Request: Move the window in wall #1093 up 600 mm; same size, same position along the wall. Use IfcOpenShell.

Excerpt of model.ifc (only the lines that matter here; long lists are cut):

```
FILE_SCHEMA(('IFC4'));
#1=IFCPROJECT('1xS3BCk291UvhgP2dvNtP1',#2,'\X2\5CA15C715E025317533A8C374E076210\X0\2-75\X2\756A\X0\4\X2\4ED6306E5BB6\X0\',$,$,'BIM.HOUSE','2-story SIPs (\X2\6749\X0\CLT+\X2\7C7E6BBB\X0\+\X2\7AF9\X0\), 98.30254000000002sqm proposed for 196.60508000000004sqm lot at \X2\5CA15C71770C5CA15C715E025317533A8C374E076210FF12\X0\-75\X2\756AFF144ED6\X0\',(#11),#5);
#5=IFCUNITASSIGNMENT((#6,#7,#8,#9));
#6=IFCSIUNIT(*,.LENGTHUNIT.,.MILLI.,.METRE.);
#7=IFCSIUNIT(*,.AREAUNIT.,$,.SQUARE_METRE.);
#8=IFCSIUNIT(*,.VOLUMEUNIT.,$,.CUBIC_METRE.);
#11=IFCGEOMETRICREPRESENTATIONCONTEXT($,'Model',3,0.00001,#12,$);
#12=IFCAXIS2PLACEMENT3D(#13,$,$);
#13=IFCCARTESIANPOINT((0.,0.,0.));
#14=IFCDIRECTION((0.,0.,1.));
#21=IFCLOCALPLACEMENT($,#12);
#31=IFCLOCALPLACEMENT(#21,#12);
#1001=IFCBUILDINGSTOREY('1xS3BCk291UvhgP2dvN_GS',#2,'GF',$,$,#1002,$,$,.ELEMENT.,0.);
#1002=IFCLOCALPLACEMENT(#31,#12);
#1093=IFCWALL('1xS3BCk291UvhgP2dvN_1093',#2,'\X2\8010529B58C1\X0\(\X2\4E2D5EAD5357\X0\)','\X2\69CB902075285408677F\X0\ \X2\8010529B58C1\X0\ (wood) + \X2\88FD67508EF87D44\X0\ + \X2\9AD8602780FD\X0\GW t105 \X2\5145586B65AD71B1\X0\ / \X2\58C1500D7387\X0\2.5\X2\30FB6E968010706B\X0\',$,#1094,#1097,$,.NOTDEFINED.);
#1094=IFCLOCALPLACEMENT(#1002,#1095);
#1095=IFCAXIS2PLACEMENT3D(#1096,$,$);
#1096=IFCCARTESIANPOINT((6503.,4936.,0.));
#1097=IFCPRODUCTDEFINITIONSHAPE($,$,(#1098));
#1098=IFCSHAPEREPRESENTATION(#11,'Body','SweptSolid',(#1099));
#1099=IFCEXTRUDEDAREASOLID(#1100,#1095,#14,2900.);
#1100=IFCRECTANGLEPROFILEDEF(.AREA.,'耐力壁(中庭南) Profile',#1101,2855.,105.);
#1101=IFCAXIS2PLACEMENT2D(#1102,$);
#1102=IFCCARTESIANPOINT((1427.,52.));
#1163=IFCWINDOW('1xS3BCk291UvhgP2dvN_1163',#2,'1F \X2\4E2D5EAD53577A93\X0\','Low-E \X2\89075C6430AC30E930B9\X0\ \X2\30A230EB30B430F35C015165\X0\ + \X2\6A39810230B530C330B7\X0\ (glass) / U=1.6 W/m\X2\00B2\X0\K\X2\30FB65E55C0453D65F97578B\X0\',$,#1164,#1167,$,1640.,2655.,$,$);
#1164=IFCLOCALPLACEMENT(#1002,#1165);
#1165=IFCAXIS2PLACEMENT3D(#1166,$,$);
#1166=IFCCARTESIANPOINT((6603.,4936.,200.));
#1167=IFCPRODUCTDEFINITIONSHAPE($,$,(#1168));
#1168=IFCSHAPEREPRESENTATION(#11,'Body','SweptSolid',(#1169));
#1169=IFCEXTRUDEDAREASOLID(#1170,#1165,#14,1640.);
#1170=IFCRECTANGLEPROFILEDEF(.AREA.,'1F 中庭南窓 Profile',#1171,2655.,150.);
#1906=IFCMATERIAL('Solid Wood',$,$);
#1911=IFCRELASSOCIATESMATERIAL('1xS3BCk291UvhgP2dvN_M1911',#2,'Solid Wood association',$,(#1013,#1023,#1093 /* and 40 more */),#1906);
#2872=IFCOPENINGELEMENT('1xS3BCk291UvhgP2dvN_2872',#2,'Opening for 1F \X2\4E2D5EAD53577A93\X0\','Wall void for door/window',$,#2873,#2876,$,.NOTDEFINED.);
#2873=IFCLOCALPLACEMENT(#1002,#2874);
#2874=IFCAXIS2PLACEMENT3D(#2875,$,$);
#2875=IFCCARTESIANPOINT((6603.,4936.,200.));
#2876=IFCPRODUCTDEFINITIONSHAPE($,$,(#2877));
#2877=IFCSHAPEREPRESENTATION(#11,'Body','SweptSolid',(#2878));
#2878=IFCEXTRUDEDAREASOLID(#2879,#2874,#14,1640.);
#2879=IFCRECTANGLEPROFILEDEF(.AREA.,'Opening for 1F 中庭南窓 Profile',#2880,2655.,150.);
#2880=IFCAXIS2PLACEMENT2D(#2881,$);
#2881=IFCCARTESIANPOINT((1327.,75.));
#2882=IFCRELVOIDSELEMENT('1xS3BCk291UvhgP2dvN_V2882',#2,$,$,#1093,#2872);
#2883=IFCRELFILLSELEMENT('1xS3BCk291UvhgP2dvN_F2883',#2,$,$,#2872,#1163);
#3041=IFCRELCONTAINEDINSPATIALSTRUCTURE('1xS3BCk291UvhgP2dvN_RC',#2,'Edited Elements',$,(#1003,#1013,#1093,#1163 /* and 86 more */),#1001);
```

```python
import numpy as np
import ifcopenshell
import ifcopenshell.api.geometry
import ifcopenshell.util.placement
import ifcopenshell.util.unit

model = ifcopenshell.open("model.ifc")
unit_scale = ifcopenshell.util.unit.calculate_unit_scale(model)

window = model.by_id(1163)
opening = window.FillsVoids[0].RelatingOpeningElement
dz = 0.6 / unit_scale

shift = np.array([0.0, 0.0, dz])
# The window is not placed relative to its opening, so move both.
for product in (opening, window):
    matrix = ifcopenshell.util.placement.get_local_placement(product.ObjectPlacement)
    matrix[:3, 3] += shift
    ifcopenshell.api.geometry.edit_object_placement(model, product=product, matrix=matrix, is_si=False)

print(f"moved by {dz * unit_scale:+.3f} m")

model.write("model_v2.ifc")
```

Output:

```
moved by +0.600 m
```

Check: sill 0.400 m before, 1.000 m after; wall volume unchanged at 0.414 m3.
